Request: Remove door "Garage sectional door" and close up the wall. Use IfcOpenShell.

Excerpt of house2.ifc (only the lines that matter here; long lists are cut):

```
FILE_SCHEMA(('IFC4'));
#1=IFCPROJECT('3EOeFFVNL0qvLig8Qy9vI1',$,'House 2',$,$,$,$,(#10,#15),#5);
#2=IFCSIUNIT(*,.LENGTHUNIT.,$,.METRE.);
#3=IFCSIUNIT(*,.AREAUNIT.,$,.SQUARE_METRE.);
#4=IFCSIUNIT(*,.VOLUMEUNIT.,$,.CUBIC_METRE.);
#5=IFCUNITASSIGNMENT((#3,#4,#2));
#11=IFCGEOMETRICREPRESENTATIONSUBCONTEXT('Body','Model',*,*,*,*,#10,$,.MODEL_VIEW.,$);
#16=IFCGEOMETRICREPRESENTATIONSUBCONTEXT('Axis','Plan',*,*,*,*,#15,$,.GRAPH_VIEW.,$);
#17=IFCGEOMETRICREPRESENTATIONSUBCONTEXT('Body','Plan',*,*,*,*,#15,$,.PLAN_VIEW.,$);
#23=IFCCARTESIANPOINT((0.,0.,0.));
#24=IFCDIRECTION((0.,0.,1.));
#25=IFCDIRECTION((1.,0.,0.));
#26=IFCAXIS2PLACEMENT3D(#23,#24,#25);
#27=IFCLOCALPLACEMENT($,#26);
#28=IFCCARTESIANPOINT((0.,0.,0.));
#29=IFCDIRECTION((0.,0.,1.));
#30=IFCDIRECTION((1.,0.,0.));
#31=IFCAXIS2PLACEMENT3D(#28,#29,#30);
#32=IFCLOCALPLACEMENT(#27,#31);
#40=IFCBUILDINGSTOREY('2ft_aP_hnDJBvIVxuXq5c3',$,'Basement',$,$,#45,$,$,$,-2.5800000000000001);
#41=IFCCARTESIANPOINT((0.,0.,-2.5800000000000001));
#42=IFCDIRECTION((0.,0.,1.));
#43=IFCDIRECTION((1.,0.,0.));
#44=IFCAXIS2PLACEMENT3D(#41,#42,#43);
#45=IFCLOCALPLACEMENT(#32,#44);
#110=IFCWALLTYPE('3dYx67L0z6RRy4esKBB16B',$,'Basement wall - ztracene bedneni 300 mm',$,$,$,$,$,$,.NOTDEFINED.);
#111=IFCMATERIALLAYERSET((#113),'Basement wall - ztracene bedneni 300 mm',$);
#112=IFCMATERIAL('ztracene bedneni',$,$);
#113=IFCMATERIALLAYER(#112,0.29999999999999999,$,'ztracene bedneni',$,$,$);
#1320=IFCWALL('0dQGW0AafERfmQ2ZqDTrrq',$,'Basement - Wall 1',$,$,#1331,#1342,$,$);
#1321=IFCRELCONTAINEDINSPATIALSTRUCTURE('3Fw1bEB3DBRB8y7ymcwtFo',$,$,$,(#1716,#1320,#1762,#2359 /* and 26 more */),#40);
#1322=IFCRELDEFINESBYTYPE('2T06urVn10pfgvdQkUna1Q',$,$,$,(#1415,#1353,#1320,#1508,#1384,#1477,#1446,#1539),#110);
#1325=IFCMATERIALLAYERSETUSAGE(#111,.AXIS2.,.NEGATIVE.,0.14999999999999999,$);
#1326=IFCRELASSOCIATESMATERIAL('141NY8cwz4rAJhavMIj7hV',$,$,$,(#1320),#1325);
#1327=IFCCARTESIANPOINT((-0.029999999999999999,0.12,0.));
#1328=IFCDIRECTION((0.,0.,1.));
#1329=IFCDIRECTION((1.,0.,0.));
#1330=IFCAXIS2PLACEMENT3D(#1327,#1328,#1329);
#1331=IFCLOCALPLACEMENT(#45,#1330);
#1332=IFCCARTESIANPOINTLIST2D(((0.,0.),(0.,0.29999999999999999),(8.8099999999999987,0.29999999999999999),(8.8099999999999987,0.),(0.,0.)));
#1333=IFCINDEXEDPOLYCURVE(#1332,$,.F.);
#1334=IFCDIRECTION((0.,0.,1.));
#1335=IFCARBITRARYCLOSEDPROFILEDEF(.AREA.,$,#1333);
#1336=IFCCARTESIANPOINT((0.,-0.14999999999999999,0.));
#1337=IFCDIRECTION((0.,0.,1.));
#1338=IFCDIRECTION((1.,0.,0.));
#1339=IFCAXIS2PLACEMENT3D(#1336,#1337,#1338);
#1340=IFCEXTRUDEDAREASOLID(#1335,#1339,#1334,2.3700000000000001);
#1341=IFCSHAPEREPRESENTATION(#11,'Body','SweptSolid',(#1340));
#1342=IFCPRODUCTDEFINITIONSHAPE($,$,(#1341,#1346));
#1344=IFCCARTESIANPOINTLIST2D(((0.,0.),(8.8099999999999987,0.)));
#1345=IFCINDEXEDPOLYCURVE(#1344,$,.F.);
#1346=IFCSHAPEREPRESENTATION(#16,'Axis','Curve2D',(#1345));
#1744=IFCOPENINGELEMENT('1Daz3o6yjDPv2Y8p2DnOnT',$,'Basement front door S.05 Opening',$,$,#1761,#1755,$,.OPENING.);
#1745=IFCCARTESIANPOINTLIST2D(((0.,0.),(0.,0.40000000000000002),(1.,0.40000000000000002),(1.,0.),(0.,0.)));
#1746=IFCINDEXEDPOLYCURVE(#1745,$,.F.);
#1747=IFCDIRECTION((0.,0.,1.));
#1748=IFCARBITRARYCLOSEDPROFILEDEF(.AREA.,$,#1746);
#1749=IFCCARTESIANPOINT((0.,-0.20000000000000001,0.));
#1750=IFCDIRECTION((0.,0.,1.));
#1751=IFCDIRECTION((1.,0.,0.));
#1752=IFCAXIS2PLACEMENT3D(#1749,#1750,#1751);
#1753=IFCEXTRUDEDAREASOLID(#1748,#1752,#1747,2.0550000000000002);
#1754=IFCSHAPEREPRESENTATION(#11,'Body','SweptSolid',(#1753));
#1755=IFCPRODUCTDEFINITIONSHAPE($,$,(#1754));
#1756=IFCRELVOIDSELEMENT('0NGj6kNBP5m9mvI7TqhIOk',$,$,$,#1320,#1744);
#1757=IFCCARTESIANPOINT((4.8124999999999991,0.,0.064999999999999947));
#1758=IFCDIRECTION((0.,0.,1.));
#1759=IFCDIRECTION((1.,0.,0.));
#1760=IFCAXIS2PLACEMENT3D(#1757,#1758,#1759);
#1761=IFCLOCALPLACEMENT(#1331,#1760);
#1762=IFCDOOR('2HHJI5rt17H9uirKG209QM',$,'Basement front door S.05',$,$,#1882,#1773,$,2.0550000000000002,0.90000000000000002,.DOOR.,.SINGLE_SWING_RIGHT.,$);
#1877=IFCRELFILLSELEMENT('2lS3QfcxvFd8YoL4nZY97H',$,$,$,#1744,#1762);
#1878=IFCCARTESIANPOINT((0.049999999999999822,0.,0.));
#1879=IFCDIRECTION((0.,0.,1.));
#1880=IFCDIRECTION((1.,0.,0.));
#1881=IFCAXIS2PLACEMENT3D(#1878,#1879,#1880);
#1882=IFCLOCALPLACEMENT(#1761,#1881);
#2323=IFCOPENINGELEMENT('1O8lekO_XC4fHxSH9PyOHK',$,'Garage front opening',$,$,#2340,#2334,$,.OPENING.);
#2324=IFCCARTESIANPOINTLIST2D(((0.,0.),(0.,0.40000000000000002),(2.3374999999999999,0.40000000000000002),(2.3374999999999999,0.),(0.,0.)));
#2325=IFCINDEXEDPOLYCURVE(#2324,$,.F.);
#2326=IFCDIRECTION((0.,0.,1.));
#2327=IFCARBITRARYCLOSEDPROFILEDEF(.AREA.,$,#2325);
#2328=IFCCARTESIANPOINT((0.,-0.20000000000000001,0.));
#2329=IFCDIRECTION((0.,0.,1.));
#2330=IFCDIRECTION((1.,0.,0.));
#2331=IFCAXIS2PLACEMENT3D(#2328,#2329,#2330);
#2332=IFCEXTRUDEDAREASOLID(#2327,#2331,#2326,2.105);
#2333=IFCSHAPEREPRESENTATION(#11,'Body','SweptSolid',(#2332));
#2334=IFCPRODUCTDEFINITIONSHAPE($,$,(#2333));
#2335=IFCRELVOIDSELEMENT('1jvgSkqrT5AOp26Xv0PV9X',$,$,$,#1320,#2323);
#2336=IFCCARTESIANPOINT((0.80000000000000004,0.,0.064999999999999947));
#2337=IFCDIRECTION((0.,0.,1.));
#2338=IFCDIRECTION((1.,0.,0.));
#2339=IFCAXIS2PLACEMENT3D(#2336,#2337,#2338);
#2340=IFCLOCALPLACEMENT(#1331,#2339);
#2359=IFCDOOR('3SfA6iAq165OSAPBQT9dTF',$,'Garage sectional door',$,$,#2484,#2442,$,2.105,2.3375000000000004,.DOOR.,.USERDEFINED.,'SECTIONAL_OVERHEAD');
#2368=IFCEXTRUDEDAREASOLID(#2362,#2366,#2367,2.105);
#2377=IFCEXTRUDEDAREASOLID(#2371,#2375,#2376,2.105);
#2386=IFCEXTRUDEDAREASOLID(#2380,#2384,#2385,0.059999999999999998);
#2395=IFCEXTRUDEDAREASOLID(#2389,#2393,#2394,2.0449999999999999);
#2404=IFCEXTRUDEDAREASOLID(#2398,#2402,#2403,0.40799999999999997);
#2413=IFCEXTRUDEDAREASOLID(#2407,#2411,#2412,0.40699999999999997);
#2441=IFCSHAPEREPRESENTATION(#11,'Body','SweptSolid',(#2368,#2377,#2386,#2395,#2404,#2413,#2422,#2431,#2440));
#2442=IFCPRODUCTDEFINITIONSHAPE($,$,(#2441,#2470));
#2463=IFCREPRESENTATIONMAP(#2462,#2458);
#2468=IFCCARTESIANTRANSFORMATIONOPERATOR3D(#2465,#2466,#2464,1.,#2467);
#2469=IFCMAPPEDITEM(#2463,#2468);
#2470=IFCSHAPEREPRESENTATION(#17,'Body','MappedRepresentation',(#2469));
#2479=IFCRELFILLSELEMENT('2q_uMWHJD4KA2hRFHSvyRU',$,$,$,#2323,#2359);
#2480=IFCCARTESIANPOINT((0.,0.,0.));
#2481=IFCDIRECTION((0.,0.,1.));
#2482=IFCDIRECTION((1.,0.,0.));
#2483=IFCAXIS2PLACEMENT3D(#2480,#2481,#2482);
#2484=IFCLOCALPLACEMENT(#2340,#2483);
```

```python
import ifcopenshell
import ifcopenshell.api.feature
import ifcopenshell.api.root
import ifcopenshell.geom
import ifcopenshell.util.shape

model = ifcopenshell.open("house2.ifc")
settings = ifcopenshell.geom.settings()


def volume(element):
    """Net volume in cubic metres, openings subtracted."""
    shape = ifcopenshell.geom.create_shape(settings, element)
    return ifcopenshell.util.shape.get_volume(shape.geometry)


door = model.by_id(2359)
opening = door.FillsVoids[0].RelatingOpeningElement
wall = opening.VoidsElements[0].RelatingBuildingElement
before = volume(wall)

ifcopenshell.api.root.remove_product(model, product=door)
ifcopenshell.api.feature.remove_feature(model, feature=opening)

after = volume(wall)

print(f"wall volume {before:.3f} -> {after:.3f} m3")

model.write("house2_updated.ifc")
```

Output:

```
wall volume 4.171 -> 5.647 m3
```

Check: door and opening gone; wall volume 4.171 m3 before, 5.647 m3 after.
